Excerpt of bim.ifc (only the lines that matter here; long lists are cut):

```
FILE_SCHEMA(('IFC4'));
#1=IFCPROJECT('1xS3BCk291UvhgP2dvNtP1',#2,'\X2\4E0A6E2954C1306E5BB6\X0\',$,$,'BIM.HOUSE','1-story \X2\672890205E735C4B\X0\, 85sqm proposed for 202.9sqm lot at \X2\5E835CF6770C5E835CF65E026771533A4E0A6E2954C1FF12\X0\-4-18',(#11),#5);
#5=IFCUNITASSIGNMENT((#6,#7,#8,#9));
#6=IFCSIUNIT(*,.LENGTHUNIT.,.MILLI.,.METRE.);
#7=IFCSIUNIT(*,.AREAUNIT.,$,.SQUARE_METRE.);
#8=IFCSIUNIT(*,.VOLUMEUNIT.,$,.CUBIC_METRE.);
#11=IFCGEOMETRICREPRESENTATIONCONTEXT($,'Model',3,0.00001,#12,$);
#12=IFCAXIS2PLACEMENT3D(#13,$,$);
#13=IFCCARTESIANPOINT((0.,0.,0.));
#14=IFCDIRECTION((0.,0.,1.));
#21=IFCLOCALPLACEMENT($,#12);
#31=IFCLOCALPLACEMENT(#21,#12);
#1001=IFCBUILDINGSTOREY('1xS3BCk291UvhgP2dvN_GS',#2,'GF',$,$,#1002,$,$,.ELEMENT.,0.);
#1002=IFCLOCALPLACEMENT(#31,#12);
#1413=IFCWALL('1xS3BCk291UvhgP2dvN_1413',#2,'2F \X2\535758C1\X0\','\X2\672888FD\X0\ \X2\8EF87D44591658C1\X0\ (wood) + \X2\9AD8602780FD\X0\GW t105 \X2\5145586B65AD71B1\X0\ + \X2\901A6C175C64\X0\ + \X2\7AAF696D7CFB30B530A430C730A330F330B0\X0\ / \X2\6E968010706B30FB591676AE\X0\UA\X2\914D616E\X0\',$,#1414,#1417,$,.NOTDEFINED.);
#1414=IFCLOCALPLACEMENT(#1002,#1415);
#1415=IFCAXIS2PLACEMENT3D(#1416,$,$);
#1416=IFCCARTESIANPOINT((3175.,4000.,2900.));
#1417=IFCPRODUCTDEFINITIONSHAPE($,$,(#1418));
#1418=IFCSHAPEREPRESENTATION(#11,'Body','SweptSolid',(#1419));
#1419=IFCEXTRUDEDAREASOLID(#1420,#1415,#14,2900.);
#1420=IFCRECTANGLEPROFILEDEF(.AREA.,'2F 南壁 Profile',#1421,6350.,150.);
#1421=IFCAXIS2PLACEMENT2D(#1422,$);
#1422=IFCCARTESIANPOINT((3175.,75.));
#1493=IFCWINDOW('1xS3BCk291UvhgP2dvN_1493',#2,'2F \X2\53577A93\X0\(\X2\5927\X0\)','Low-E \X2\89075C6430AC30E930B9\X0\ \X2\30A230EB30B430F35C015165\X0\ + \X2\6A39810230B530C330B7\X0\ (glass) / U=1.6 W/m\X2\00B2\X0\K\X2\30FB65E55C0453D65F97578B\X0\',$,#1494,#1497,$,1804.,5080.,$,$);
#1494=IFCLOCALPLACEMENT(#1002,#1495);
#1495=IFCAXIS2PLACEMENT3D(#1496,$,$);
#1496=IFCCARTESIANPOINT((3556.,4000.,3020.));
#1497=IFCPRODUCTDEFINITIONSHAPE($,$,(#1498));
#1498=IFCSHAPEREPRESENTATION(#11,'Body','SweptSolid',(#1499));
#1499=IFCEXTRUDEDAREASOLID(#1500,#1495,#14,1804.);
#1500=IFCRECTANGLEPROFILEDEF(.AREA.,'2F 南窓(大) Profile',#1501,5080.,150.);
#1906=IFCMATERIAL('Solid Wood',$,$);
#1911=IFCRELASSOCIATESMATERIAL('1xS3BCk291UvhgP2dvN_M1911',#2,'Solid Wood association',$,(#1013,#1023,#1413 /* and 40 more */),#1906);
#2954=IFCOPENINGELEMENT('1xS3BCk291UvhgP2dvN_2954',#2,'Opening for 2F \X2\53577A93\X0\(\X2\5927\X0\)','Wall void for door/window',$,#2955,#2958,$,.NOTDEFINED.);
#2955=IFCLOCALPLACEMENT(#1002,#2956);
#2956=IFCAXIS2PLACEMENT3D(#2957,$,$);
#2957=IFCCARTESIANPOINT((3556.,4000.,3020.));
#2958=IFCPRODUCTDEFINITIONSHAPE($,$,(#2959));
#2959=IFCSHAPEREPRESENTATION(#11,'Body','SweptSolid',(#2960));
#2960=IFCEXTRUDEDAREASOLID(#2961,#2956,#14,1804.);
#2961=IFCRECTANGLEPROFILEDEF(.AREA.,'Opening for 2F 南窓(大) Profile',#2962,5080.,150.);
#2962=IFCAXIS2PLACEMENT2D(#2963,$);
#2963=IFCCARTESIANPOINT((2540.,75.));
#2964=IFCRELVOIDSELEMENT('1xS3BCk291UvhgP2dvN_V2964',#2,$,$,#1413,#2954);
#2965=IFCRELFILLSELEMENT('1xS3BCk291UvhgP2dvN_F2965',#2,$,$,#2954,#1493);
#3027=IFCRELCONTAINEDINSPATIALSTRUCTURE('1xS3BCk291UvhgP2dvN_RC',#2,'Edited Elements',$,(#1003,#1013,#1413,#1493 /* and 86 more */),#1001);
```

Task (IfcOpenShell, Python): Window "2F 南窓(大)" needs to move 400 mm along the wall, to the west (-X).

```python
import ifcopenshell
import ifcopenshell.api.geometry
import ifcopenshell.util.placement

model = ifcopenshell.open("bim.ifc")

window = model.by_id(1493)
opening = window.FillsVoids[0].RelatingOpeningElement
wall = opening.VoidsElements[0].RelatingBuildingElement

wall_matrix = ifcopenshell.util.placement.get_local_placement(wall.ObjectPlacement)
shift = wall_matrix[:3, 0] * -400.0
before = ifcopenshell.util.placement.get_local_placement(window.ObjectPlacement)[:3, 3].copy()

# The window is not placed relative to its opening, so move both.
for product in (opening, window):
    matrix = ifcopenshell.util.placement.get_local_placement(product.ObjectPlacement)
    matrix[:3, 3] += shift
    ifcopenshell.api.geometry.edit_object_placement(model, product=product, matrix=matrix, is_si=False)

after = ifcopenshell.util.placement.get_local_placement(window.ObjectPlacement)[:3, 3]
print("window moved by", (after - before).round(3) + 0.0)

model.write("bim-out.ifc")
```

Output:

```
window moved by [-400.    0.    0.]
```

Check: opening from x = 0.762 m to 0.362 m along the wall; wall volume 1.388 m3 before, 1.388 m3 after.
